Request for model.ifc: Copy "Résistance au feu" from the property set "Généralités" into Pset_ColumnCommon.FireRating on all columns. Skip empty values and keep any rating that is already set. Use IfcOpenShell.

First a look at what the model holds.

```python
import ifcopenshell
import ifcopenshell.util.element

model = ifcopenshell.open("model.ifc")
print(model.schema)
columns = model.by_type("IfcColumn")
print(len(columns), "columns")
for e in columns[:8]:
    source = ifcopenshell.util.element.get_pset(e, "Généralités", "Résistance au feu")
    target = ifcopenshell.util.element.get_pset(e, "Pset_ColumnCommon", "FireRating")
    print(e.id(), repr(source), repr(target), sep=" | ")
```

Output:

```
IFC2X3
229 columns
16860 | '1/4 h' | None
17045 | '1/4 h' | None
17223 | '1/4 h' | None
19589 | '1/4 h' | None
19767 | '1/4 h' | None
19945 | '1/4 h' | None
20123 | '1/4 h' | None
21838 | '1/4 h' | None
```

```python
import ifcopenshell
import ifcopenshell.api.pset
import ifcopenshell.util.element

model = ifcopenshell.open("model.ifc")

count = 0
for e in model.by_type("IfcColumn"):
    value = ifcopenshell.util.element.get_pset(e, "Généralités", "Résistance au feu")
    current = ifcopenshell.util.element.get_pset(e, "Pset_ColumnCommon", "FireRating")
    if not value or not value.strip() or current:
        continue
    # add_pset returns the element's existing set when there is one.
    pset = ifcopenshell.api.pset.add_pset(model, product=e, name="Pset_ColumnCommon")
    ifcopenshell.api.pset.edit_pset(model, pset=pset, properties={"FireRating": value})
    count += 1

print(count, "columns updated")

model.write("model_v2.ifc")
```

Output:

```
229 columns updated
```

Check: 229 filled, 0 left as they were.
